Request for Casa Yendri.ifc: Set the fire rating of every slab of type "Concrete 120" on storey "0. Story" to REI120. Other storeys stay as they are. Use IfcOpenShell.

First a look at what the model holds.

```python
import ifcopenshell
import ifcopenshell.util.element

model = ifcopenshell.open("Casa Yendri.ifc")
print(model.schema)
storey = next(s for s in model.by_type("IfcBuildingStorey") if s.Name == "0. Story")
slabs = [e for e in ifcopenshell.util.element.get_decomposition(storey) if e.is_a("IfcSlab")]
seen = {}
for e in slabs:
    element_type = ifcopenshell.util.element.get_type(e)
    key = (element_type.Name if element_type != e and element_type else None, ifcopenshell.util.element.get_pset(e, "Pset_SlabCommon", "FireRating"))
    seen[key] = seen.get(key, 0) + 1
for (name, value), count in sorted(seen.items(), key=str):
    print(count, "x", name, "|", value)
```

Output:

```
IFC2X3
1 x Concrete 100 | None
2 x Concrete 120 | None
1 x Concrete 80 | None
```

```python
import ifcopenshell
import ifcopenshell.api.pset
import ifcopenshell.util.element

model = ifcopenshell.open("Casa Yendri.ifc")

storey = next(s for s in model.by_type("IfcBuildingStorey") if s.Name == "0. Story")
slabs = [e for e in ifcopenshell.util.element.get_decomposition(storey) if e.is_a("IfcSlab")]

count = 0
for e in slabs:
    element_type = ifcopenshell.util.element.get_type(e)
    if element_type in (None, e) or element_type.Name != "Concrete 120":
        continue
    # add_pset returns the element's existing set when there is one.
    pset = ifcopenshell.api.pset.add_pset(model, product=e, name="Pset_SlabCommon")
    ifcopenshell.api.pset.edit_pset(model, pset=pset, properties={"FireRating": "REI120"})
    count += 1

print(count, "slabs updated")

model.write("Casa Yendri_updated.ifc")
```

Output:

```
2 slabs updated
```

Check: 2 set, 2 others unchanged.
